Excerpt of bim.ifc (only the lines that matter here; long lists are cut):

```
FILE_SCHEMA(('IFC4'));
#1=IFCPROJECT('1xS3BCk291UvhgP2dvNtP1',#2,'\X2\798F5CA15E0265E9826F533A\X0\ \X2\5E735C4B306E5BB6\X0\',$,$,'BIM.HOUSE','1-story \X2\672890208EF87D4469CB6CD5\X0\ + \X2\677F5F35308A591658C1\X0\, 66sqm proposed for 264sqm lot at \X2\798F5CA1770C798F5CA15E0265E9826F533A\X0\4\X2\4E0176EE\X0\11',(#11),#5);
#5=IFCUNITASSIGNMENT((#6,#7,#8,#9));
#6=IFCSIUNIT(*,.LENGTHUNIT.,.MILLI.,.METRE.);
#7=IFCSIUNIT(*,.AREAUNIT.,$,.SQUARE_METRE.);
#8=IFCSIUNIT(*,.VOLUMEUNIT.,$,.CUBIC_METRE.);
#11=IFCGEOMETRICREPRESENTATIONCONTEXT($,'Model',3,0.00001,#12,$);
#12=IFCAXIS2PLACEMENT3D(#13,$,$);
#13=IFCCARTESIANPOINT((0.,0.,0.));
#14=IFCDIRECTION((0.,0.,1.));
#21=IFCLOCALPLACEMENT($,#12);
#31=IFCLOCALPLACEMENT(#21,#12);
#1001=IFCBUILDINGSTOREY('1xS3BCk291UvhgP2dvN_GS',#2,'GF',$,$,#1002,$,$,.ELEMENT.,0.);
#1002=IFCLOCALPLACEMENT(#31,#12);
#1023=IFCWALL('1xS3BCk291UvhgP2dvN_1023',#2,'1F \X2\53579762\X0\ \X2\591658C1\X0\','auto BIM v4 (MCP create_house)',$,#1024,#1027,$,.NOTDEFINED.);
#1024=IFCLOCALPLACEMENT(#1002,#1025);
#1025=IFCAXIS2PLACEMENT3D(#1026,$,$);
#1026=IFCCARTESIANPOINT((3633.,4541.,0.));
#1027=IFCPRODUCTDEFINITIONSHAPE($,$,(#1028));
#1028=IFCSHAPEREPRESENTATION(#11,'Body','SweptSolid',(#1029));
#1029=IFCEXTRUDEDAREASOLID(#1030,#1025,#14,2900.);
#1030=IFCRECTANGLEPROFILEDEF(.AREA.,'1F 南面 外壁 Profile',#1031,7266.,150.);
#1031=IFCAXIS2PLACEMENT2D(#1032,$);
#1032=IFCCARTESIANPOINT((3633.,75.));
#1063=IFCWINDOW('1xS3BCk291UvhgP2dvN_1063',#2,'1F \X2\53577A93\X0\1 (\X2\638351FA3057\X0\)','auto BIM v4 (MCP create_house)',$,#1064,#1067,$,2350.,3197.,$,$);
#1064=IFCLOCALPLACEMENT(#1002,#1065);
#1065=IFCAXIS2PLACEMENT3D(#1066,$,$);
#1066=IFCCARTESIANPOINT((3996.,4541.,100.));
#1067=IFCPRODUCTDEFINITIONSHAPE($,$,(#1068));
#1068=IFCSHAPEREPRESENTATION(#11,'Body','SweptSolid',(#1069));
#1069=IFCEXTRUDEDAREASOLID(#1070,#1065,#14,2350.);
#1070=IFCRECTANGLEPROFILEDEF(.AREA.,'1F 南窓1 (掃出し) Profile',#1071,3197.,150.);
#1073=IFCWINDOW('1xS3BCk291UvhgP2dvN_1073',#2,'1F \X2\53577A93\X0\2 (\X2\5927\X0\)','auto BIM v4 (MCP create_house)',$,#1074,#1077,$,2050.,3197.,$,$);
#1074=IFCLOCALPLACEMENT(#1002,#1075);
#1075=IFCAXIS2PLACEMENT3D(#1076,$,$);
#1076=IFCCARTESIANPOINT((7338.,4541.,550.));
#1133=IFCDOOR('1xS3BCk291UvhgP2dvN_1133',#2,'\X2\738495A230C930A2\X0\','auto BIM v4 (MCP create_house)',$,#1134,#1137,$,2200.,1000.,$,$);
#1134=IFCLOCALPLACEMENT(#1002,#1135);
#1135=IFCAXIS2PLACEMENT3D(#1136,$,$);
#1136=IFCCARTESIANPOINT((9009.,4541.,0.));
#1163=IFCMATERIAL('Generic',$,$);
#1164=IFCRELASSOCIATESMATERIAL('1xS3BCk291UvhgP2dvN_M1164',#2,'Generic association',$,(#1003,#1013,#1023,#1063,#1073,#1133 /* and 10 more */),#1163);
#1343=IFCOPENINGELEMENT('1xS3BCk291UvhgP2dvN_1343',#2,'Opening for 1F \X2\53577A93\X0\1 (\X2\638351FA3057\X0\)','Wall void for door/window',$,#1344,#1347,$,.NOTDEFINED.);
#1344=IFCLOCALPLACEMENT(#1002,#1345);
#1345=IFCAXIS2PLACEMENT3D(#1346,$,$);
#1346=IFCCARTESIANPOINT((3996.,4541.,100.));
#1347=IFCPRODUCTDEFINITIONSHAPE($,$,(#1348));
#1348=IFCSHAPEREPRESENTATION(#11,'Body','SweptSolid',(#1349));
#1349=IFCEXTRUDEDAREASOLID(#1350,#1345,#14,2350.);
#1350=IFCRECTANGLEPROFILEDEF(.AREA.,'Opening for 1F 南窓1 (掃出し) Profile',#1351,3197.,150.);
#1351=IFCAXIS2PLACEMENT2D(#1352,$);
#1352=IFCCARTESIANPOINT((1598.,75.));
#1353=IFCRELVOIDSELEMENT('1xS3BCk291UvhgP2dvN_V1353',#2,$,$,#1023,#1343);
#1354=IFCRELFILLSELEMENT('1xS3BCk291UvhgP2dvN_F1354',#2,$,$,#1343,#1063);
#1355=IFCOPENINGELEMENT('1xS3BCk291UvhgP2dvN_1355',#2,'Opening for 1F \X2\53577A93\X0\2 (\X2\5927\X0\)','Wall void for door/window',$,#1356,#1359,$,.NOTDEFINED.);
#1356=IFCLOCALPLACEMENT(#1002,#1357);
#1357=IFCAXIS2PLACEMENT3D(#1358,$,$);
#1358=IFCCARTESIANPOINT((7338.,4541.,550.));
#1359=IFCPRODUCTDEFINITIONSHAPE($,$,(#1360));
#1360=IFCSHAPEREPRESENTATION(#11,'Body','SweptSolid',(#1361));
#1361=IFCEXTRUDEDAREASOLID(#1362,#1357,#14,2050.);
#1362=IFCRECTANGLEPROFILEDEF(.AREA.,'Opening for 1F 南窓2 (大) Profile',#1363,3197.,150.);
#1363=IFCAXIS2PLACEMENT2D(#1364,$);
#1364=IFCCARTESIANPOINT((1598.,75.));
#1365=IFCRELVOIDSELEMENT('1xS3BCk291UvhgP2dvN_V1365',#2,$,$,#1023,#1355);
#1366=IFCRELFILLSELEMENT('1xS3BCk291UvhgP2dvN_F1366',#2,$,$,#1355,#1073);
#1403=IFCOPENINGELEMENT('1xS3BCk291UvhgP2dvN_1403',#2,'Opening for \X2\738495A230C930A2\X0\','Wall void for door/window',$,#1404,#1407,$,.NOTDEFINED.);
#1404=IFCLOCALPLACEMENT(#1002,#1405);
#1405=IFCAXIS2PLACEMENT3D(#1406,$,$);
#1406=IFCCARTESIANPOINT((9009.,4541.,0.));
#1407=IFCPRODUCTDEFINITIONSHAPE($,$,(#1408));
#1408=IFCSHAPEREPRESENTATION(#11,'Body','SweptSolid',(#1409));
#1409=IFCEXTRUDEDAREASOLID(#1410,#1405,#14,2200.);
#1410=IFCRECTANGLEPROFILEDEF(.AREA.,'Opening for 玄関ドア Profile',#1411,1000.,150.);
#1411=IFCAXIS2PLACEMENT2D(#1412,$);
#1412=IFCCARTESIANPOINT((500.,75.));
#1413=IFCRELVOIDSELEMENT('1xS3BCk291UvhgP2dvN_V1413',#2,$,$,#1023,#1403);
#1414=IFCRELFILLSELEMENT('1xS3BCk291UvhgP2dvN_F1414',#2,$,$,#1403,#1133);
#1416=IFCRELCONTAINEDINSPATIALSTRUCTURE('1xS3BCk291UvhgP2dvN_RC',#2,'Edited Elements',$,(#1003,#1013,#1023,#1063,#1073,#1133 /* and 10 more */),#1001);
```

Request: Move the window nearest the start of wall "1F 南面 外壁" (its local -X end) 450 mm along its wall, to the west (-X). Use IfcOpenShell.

```python
import ifcopenshell
import ifcopenshell.api.geometry
import ifcopenshell.util.placement
import ifcopenshell.util.unit

model = ifcopenshell.open("bim.ifc")
unit_scale = ifcopenshell.util.unit.calculate_unit_scale(model)

window = model.by_guid("1xS3BCk291UvhgP2dvN_1063")
opening = window.FillsVoids[0].RelatingOpeningElement
wall = opening.VoidsElements[0].RelatingBuildingElement

wall_matrix = ifcopenshell.util.placement.get_local_placement(wall.ObjectPlacement)
shift = wall_matrix[:3, 0] * -0.45 / unit_scale
before = ifcopenshell.util.placement.get_local_placement(window.ObjectPlacement)[:3, 3].copy()

# The window is not placed relative to its opening, so move both.
for product in (opening, window):
    matrix = ifcopenshell.util.placement.get_local_placement(product.ObjectPlacement)
    matrix[:3, 3] += shift
    ifcopenshell.api.geometry.edit_object_placement(model, product=product, matrix=matrix, is_si=False)

after = ifcopenshell.util.placement.get_local_placement(window.ObjectPlacement)[:3, 3]
print("window moved by", (after - before).round(3) + 0.0)

model.write("bim_rev.ifc")
```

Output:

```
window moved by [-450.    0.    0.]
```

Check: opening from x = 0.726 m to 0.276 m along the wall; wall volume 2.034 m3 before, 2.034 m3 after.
